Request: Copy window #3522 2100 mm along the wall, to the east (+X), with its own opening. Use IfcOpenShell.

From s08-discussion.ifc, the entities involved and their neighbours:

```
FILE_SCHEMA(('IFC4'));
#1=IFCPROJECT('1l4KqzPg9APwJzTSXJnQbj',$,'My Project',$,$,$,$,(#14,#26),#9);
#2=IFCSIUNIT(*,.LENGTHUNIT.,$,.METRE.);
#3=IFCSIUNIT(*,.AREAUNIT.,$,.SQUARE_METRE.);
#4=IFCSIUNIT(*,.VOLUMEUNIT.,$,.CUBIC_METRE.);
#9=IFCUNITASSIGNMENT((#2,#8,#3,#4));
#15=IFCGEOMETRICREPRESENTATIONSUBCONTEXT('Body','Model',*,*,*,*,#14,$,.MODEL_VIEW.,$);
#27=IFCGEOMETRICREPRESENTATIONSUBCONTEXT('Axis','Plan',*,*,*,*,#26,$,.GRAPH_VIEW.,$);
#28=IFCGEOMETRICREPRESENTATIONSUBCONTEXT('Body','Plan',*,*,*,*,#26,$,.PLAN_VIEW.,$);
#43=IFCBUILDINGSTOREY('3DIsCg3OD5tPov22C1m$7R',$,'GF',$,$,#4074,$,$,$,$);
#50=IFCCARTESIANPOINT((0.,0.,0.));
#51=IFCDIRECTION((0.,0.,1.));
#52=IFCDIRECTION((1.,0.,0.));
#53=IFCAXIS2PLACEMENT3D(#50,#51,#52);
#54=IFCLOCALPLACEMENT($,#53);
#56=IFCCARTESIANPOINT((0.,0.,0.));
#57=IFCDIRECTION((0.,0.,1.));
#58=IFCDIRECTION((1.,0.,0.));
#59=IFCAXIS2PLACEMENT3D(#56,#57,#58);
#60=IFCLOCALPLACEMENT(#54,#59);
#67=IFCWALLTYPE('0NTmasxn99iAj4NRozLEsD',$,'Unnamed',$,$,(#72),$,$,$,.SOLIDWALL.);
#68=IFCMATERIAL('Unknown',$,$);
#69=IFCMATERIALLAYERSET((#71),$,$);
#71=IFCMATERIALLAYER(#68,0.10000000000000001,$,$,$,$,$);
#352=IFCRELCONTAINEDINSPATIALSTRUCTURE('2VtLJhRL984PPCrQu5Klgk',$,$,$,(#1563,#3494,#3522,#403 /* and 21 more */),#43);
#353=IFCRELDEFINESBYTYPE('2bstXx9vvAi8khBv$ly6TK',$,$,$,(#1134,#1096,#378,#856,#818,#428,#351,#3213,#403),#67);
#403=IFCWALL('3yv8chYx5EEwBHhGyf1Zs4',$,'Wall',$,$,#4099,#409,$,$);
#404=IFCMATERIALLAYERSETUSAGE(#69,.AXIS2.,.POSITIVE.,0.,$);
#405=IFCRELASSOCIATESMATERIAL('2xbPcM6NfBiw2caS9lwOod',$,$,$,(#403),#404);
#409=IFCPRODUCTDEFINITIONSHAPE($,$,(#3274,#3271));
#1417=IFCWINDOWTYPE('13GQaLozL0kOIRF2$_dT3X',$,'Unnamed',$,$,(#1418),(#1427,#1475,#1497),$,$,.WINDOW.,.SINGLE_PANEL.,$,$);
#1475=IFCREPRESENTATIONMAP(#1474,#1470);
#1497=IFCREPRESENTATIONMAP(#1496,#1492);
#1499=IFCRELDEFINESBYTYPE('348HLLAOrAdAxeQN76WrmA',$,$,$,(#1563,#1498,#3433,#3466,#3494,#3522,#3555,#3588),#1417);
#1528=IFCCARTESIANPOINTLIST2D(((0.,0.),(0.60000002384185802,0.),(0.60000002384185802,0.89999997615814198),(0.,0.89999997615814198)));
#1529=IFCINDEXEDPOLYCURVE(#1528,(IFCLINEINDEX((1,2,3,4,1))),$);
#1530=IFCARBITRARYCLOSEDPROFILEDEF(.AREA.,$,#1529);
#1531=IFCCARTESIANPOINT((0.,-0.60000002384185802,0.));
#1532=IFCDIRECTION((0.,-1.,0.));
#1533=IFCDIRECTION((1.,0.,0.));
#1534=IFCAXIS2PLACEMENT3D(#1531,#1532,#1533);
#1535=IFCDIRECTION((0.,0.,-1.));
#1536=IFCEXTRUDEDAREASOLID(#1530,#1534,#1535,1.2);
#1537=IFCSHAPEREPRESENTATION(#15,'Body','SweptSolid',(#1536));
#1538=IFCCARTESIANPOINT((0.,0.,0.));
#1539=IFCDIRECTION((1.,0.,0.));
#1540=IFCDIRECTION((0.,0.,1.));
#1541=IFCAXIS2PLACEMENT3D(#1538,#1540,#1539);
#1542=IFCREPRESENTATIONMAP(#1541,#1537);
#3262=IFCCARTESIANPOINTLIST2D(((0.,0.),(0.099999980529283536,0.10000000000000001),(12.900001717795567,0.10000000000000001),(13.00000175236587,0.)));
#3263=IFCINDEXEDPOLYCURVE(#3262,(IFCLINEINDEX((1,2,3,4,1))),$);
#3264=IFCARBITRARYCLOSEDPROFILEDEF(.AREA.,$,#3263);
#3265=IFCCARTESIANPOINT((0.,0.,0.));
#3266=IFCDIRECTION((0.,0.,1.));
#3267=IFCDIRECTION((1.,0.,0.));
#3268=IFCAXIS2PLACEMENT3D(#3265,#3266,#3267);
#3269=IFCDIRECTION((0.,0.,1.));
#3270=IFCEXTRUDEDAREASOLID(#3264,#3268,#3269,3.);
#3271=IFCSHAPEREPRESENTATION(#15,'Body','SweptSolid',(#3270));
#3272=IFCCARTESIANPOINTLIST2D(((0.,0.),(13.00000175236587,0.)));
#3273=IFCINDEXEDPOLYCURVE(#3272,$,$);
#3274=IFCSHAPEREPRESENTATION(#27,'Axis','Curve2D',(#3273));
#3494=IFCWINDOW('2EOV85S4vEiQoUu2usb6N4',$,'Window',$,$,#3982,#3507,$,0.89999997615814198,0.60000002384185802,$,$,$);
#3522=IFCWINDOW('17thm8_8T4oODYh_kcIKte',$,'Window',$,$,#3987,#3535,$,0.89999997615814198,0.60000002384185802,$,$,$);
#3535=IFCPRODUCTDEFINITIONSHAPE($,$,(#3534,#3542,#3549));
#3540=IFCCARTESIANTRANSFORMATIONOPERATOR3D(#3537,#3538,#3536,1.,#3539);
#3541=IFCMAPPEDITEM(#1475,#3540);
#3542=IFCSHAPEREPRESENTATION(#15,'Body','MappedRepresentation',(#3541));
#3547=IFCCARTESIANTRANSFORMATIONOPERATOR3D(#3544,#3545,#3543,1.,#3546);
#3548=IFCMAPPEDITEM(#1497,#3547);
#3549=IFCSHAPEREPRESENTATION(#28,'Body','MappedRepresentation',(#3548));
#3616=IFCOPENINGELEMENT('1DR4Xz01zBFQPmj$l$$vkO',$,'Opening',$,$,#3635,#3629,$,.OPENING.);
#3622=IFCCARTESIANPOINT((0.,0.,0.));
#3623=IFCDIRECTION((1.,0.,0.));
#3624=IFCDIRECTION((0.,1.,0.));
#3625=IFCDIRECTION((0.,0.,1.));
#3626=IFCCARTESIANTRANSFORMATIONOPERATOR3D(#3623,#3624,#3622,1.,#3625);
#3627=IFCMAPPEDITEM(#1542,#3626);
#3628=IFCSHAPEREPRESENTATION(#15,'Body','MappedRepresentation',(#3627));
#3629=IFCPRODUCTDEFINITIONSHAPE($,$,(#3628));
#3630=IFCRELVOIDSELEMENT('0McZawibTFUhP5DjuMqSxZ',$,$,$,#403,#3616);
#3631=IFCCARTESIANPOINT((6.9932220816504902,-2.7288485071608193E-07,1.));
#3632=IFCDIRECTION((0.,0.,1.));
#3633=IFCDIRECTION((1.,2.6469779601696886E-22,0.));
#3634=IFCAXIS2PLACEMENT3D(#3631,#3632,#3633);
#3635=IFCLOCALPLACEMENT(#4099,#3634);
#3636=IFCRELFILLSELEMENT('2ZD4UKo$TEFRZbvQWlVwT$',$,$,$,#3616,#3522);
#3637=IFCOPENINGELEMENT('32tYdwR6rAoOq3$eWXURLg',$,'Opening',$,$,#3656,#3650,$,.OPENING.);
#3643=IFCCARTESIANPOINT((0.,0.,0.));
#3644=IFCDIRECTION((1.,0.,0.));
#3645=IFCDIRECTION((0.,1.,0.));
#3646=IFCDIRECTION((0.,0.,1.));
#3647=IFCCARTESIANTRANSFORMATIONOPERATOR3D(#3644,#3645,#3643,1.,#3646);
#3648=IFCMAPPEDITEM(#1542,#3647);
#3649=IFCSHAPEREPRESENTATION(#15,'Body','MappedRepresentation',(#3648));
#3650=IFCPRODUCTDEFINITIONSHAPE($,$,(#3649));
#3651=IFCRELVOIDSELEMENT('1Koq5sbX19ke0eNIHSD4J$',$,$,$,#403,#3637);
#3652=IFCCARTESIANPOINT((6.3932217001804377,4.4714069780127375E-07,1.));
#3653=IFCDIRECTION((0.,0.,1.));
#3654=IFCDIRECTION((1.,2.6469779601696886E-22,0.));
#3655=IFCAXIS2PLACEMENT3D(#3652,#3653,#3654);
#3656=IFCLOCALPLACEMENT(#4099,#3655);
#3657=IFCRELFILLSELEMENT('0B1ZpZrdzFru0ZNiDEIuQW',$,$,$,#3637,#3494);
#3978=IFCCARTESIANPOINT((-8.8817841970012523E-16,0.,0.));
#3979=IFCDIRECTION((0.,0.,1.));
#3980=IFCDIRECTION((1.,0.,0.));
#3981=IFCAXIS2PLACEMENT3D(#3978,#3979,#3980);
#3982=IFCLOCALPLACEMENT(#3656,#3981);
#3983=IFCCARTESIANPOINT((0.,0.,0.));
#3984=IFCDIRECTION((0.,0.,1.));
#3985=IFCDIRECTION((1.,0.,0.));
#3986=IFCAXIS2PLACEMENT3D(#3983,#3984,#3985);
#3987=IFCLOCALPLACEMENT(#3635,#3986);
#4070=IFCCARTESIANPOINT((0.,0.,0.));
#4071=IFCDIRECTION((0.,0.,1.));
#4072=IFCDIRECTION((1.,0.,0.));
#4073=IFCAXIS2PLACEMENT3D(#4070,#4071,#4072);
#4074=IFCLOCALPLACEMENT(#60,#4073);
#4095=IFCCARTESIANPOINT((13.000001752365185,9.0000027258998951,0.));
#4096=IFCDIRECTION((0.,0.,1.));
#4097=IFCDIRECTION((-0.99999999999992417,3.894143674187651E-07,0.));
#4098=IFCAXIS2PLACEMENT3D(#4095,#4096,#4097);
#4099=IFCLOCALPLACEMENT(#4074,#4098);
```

```python
import ifcopenshell
import ifcopenshell.api.feature
import ifcopenshell.api.geometry
import ifcopenshell.api.root
import ifcopenshell.geom
import ifcopenshell.util.element
import ifcopenshell.util.placement
import ifcopenshell.util.shape
import ifcopenshell.util.unit

model = ifcopenshell.open("s08-discussion.ifc")
unit_scale = ifcopenshell.util.unit.calculate_unit_scale(model)
settings = ifcopenshell.geom.settings()


def volume(element):
    """Net volume in cubic metres, openings subtracted."""
    shape = ifcopenshell.geom.create_shape(settings, element)
    return ifcopenshell.util.shape.get_volume(shape.geometry)


window = model.by_id(3522)
opening = window.FillsVoids[0].RelatingOpeningElement
wall = opening.VoidsElements[0].RelatingBuildingElement
before = volume(wall)
shift = ifcopenshell.util.placement.get_local_placement(wall.ObjectPlacement)[:3, 0] * -2.1 / unit_scale

# copy_class copies the void relationship, type, container and properties, but no geometry.
new_opening = ifcopenshell.api.root.copy_class(model, product=opening)
new_opening.Representation = ifcopenshell.util.element.copy_deep(
    model, opening.Representation, exclude=["IfcGeometricRepresentationContext", "IfcRepresentationMap"]
)
new_window = ifcopenshell.api.root.copy_class(model, product=window)
new_window.Representation = ifcopenshell.util.element.copy_deep(
    model, window.Representation, exclude=["IfcGeometricRepresentationContext", "IfcRepresentationMap"]
)
ifcopenshell.api.feature.add_filling(model, opening=new_opening, element=new_window)

for old, new in ((opening, new_opening), (window, new_window)):
    matrix = ifcopenshell.util.placement.get_local_placement(old.ObjectPlacement)
    matrix[:3, 3] += shift
    ifcopenshell.api.geometry.edit_object_placement(model, product=new, matrix=matrix, is_si=False)

after = volume(wall)

print(f"wall volume {before:.3f} -> {after:.3f} m3")

model.write("s08-discussion_updated.ifc")
```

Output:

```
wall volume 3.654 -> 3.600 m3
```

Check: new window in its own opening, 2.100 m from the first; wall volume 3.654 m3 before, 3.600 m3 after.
